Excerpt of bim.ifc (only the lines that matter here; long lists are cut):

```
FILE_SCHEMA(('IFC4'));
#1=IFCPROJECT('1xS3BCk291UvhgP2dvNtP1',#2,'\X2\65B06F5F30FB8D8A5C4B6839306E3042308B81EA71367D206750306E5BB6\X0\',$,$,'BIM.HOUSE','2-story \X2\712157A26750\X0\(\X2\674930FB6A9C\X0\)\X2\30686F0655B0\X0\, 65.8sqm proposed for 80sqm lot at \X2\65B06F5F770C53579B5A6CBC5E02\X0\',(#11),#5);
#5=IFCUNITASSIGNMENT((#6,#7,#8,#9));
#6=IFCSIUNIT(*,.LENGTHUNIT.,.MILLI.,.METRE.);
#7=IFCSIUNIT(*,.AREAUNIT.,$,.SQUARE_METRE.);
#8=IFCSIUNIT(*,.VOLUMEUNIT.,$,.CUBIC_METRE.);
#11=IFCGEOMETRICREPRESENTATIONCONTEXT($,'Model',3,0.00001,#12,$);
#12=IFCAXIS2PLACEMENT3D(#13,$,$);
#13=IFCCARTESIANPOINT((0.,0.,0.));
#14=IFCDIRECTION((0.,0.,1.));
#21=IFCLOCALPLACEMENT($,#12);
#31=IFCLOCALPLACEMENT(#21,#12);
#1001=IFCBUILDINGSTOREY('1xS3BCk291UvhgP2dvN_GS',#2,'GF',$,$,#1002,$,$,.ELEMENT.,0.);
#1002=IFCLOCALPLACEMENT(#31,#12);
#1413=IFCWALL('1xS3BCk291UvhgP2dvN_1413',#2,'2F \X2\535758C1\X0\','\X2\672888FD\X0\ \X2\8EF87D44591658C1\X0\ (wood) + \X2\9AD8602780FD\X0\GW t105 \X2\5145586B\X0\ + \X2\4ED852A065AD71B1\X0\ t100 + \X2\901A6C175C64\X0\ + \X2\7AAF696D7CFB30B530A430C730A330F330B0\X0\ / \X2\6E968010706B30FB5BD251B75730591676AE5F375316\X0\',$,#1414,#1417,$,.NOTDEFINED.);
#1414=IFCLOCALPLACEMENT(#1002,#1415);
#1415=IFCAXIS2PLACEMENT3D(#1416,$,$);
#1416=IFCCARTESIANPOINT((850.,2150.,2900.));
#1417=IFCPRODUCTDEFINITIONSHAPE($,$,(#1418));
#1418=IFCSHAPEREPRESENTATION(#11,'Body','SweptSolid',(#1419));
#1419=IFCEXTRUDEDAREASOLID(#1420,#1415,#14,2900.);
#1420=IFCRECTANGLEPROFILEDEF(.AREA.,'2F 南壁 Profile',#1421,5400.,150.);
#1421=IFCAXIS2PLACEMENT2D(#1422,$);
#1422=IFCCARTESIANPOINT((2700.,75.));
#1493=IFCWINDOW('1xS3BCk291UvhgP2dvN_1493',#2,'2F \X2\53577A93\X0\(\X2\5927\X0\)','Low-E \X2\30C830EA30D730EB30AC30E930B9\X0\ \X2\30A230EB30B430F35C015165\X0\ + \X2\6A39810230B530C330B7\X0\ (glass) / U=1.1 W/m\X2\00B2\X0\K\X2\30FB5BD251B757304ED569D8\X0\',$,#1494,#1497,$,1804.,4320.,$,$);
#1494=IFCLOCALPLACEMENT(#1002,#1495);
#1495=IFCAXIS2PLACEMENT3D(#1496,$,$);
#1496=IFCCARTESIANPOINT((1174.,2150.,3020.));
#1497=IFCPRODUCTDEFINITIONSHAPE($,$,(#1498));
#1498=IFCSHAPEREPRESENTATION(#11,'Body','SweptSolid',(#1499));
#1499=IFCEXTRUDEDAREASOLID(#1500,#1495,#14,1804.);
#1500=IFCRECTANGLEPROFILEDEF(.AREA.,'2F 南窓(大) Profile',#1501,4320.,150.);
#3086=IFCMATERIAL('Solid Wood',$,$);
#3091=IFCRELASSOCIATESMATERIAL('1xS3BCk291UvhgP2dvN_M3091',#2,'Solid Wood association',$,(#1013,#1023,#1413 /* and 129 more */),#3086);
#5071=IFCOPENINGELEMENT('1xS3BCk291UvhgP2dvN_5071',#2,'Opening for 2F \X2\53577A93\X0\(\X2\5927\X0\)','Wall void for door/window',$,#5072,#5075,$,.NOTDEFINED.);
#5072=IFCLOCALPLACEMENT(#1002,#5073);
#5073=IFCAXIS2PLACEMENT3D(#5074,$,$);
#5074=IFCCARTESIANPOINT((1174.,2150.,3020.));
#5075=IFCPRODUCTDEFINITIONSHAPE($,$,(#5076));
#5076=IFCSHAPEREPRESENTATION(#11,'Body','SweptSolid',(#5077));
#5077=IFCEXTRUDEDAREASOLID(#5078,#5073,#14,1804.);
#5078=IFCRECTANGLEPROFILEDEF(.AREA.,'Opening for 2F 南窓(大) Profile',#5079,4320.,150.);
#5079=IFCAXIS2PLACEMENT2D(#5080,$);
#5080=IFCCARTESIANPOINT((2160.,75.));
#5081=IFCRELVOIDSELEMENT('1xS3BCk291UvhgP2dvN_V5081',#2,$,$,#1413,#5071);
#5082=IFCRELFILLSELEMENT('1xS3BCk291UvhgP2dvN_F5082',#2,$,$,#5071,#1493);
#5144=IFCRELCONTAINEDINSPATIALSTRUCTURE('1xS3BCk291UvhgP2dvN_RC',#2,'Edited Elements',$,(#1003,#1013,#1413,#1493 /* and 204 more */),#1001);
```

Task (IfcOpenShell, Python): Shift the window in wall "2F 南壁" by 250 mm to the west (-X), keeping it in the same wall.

```python
import ifcopenshell
import ifcopenshell.api.geometry
import ifcopenshell.util.placement
import ifcopenshell.util.unit

model = ifcopenshell.open("bim.ifc")
unit_scale = ifcopenshell.util.unit.calculate_unit_scale(model)

window = model.by_guid("1xS3BCk291UvhgP2dvN_1493")
opening = window.FillsVoids[0].RelatingOpeningElement
wall = opening.VoidsElements[0].RelatingBuildingElement

wall_matrix = ifcopenshell.util.placement.get_local_placement(wall.ObjectPlacement)
shift = wall_matrix[:3, 0] * -0.25 / unit_scale
before = ifcopenshell.util.placement.get_local_placement(window.ObjectPlacement)[:3, 3].copy()

# The window is not placed relative to its opening, so move both.
for product in (opening, window):
    matrix = ifcopenshell.util.placement.get_local_placement(product.ObjectPlacement)
    matrix[:3, 3] += shift
    ifcopenshell.api.geometry.edit_object_placement(model, product=product, matrix=matrix, is_si=False)

after = ifcopenshell.util.placement.get_local_placement(window.ObjectPlacement)[:3, 3]
print("window moved by", (after - before).round(3) + 0.0)

model.write("bim_updated.ifc")
```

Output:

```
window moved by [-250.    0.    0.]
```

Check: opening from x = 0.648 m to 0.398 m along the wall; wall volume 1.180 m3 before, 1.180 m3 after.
